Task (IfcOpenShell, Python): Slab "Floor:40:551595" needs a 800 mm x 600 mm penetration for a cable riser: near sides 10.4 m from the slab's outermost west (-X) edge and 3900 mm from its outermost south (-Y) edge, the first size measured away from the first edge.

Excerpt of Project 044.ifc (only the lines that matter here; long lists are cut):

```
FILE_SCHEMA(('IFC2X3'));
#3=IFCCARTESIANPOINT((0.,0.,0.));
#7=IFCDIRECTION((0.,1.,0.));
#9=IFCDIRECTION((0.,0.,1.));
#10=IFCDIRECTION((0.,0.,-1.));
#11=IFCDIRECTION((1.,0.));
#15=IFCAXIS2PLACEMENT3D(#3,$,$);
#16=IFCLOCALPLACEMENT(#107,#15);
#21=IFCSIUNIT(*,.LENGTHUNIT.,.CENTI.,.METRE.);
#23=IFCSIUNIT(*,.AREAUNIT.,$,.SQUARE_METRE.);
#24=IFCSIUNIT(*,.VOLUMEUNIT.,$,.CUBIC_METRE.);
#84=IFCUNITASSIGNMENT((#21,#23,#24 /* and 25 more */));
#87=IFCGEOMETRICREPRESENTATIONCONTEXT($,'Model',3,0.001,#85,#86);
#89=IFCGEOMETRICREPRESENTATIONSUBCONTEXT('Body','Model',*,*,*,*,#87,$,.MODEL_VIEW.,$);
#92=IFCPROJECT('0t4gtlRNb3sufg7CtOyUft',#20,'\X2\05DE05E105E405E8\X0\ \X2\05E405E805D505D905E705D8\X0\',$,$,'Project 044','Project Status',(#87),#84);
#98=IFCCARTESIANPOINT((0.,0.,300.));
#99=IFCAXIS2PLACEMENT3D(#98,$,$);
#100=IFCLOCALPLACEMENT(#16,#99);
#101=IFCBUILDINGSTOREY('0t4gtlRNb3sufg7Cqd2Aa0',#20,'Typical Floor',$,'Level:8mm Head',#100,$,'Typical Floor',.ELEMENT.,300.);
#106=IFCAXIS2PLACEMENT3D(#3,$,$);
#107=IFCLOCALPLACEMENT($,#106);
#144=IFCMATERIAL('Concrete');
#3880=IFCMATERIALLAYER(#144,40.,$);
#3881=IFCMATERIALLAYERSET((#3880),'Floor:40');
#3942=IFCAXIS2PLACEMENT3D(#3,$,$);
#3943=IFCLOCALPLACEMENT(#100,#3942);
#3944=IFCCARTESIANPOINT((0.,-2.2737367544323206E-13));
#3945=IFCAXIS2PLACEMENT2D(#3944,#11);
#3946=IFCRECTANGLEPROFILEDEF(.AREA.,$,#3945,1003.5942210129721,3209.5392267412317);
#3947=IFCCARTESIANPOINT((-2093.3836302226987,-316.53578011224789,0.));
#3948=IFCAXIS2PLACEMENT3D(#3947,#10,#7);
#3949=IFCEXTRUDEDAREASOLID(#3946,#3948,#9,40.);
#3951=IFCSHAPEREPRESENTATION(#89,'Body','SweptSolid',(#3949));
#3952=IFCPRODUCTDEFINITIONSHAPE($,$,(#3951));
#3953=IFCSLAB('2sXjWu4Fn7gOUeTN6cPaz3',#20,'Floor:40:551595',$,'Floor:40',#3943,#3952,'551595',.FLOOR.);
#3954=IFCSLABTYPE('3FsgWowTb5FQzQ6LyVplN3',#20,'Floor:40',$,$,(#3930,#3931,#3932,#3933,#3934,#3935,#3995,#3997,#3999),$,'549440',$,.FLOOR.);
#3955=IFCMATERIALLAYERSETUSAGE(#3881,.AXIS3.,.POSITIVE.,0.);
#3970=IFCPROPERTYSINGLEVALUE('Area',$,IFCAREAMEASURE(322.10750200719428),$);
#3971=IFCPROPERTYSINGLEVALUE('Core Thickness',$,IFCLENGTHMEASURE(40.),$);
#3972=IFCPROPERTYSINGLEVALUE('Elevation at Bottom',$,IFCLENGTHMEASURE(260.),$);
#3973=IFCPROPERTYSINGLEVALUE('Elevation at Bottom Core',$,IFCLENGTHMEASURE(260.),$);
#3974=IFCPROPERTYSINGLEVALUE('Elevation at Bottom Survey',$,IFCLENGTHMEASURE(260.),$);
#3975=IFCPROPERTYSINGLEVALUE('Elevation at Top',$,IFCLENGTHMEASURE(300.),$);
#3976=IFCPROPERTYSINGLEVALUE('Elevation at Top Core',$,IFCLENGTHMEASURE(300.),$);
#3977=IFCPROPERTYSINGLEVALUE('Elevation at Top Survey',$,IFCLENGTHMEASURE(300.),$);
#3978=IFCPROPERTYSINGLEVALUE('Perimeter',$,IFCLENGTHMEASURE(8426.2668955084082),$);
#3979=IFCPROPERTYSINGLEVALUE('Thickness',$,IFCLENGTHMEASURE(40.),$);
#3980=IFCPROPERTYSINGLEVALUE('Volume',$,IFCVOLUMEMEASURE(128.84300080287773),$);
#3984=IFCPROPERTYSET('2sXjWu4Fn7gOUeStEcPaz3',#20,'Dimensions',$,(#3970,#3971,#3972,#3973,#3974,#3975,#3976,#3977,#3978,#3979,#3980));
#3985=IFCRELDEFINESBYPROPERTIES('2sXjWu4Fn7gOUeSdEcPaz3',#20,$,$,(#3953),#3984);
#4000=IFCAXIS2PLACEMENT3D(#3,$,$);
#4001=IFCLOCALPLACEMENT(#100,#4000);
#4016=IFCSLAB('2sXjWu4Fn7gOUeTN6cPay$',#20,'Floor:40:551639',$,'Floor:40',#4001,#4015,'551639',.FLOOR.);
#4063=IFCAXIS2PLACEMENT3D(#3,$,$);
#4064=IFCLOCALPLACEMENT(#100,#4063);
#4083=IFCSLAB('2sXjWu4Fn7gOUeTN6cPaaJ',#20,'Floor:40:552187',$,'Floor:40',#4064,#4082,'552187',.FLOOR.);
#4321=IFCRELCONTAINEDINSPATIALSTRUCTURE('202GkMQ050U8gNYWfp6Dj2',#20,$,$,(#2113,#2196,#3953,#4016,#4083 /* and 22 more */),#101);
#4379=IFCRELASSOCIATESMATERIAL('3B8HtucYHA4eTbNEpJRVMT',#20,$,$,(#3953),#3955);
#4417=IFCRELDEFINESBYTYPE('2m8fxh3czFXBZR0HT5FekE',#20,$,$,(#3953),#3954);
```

```python
import numpy as np
import ifcopenshell
import ifcopenshell.api.feature
import ifcopenshell.api.geometry
import ifcopenshell.api.pset
import ifcopenshell.api.root
import ifcopenshell.geom
import ifcopenshell.util.element
import ifcopenshell.util.placement
import ifcopenshell.util.representation
import ifcopenshell.util.shape
import ifcopenshell.util.unit

model = ifcopenshell.open("Project 044.ifc")
unit_scale = ifcopenshell.util.unit.calculate_unit_scale(model)
area_scale = ifcopenshell.util.unit.calculate_unit_scale(model, "AREAUNIT")
volume_scale = ifcopenshell.util.unit.calculate_unit_scale(model, "VOLUMEUNIT")
settings = ifcopenshell.geom.settings()


def volume(element):
    """Net volume in cubic metres, openings subtracted."""
    shape = ifcopenshell.geom.create_shape(settings, element)
    return ifcopenshell.util.shape.get_volume(shape.geometry)


slab = model.by_guid("2sXjWu4Fn7gOUeTN6cPaz3")
before = volume(slab)

# Extent in the slab's own axes, in metres. The edges named are its -X and -Y sides.
slab_shape = ifcopenshell.geom.create_shape(settings, slab)
vertices = ifcopenshell.util.shape.get_vertices(slab_shape.geometry)
x_min, y_min, bottom = vertices.min(axis=0)
top = vertices[:, 2].max()

opening = ifcopenshell.api.root.create_entity(model, ifc_class="IfcOpeningElement", name="Cable riser opening")
context = ifcopenshell.util.representation.get_context(model, "Model", "Body", "MODEL_VIEW")
width, depth = 0.8, 0.6
outline = [(0.0, 0.0), (width, 0.0), (width, depth), (0.0, depth), (0.0, 0.0)]
# Overshoot both faces by 50 mm so the cut is clean.
shape = ifcopenshell.api.geometry.add_slab_representation(
    model, context=context, depth=top - bottom + 0.1, polyline=outline
)
ifcopenshell.api.geometry.assign_representation(model, product=opening, representation=shape)

matrix = ifcopenshell.util.placement.get_local_placement(slab.ObjectPlacement)
matrix[:, 3] = matrix @ np.append(np.array([x_min + 10.4, y_min + 3.9, bottom - 0.05]) / unit_scale, 1.0)
ifcopenshell.api.geometry.edit_object_placement(model, product=opening, matrix=matrix, is_si=False)
ifcopenshell.api.feature.add_feature(model, feature=opening, element=slab)

after = volume(slab)

# Update the slab's stored quantities.
pset = model.by_id(ifcopenshell.util.element.get_pset(slab, "Dimensions", should_inherit=False)["id"])
ifcopenshell.api.pset.edit_pset(model, pset=pset, properties={
    "Area": model.create_entity("IfcAreaMeasure", after / (top - bottom) / area_scale),
    "Volume": model.create_entity("IfcVolumeMeasure", after / volume_scale),
})

print(f"slab volume {before:.3f} -> {after:.3f} m3")

model.write("Project 044_updated.ifc")
```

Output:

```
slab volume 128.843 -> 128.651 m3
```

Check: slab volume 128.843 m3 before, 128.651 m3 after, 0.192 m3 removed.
